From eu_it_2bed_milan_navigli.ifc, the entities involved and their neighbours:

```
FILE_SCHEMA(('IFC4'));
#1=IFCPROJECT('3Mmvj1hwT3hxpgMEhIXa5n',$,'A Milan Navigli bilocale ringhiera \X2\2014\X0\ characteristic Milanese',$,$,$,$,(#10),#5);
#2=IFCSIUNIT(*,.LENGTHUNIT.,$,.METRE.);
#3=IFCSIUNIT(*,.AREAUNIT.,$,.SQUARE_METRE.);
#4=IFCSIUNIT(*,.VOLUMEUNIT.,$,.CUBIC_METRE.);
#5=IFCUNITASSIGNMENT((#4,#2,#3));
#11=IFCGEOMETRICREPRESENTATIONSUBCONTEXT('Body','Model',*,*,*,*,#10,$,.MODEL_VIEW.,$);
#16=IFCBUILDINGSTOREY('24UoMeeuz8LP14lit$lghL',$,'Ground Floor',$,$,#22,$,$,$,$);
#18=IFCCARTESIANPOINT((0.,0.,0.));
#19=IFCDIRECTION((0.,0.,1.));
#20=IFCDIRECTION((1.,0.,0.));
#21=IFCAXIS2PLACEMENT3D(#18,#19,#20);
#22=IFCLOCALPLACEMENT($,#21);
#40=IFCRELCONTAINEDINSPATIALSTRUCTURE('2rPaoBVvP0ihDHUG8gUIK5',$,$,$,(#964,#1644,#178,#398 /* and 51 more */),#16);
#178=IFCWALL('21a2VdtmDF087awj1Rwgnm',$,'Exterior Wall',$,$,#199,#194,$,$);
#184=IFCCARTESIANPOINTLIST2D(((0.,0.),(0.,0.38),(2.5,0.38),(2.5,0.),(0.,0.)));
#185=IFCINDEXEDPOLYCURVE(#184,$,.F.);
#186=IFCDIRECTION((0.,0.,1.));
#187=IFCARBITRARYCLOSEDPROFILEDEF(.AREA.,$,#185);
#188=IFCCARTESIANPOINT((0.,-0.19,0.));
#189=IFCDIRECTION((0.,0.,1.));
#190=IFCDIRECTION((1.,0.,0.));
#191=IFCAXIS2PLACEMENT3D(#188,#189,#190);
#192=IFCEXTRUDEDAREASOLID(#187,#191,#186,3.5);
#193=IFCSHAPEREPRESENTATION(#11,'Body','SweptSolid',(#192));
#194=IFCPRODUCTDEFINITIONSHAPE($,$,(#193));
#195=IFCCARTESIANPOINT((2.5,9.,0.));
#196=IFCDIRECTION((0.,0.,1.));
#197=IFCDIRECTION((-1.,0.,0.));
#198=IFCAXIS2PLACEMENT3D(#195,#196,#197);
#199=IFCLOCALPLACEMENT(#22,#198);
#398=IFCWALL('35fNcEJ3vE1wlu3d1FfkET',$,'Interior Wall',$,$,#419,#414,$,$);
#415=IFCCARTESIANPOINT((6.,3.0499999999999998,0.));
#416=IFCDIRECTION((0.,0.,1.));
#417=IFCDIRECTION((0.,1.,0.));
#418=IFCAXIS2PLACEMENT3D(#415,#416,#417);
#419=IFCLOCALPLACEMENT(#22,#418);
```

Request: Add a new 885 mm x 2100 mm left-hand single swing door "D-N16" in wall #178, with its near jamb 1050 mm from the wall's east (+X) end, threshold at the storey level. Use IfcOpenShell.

```python
import numpy as np
import ifcopenshell
import ifcopenshell.api.feature
import ifcopenshell.api.geometry
import ifcopenshell.api.root
import ifcopenshell.api.spatial
import ifcopenshell.geom
import ifcopenshell.util.element
import ifcopenshell.util.placement
import ifcopenshell.util.representation
import ifcopenshell.util.shape
import ifcopenshell.util.unit

model = ifcopenshell.open("eu_it_2bed_milan_navigli.ifc")
unit_scale = ifcopenshell.util.unit.calculate_unit_scale(model)
settings = ifcopenshell.geom.settings()


def volume(element):
    """Net volume in cubic metres, openings subtracted."""
    shape = ifcopenshell.geom.create_shape(settings, element)
    return ifcopenshell.util.shape.get_volume(shape.geometry)


wall = model.by_id(178)
storey = ifcopenshell.util.element.get_container(wall, ifc_class="IfcBuildingStorey")
context = ifcopenshell.util.representation.get_context(model, "Model", "Body", "MODEL_VIEW")
before = volume(wall)

width, height, from_end, sill = 0.885, 2.1, 1.05, 0.0  # metres

# The wall runs along its own X axis, and the end named is its -X end.
wall_shape = ifcopenshell.geom.create_shape(settings, wall)
x, y, z = ifcopenshell.util.shape.get_vertices(wall_shape.geometry).T
start = x.min() + from_end
face, thickness = float(y.min()), float(y.max() - y.min())
wall_matrix = ifcopenshell.util.placement.get_local_placement(wall.ObjectPlacement)
level = ifcopenshell.util.placement.get_local_placement(storey.ObjectPlacement)[2, 3]


def in_wall(x, y):
    """Placement at x, y metres in the wall's axes, at sill height."""
    matrix = wall_matrix.copy()
    matrix[:, 3] = wall_matrix @ np.array([x / unit_scale, y / unit_scale, 0.0, 1.0])
    matrix[2, 3] = level + sill / unit_scale
    return matrix


# Opening: a box that overshoots both wall faces by 50 mm.
opening = ifcopenshell.api.root.create_entity(model, ifc_class="IfcOpeningElement", predefined_type="OPENING")
box = ifcopenshell.api.geometry.add_wall_representation(
    model, context=context, length=width, height=height, thickness=thickness + 0.1
)
ifcopenshell.api.geometry.assign_representation(model, product=opening, representation=box)
ifcopenshell.api.geometry.edit_object_placement(model, product=opening, matrix=in_wall(start, face - 0.05), is_si=False)
ifcopenshell.api.feature.add_feature(model, feature=opening, element=wall)

door = ifcopenshell.api.root.create_entity(model, ifc_class="IfcDoor", name="D-N16", predefined_type="DOOR")
door.OverallWidth, door.OverallHeight = width / unit_scale, height / unit_scale
door.OperationType = "SINGLE_SWING_LEFT"
body = ifcopenshell.api.geometry.add_door_representation(
    model,
    context=context,
    overall_width=door.OverallWidth,
    overall_height=door.OverallHeight,
    operation_type="SINGLE_SWING_LEFT",
    lining_properties={"LiningDepth": thickness / unit_scale, "ThresholdDepth": thickness / unit_scale},
)
ifcopenshell.api.geometry.assign_representation(model, product=door, representation=body)
ifcopenshell.api.spatial.assign_container(model, products=[door], relating_structure=storey)
ifcopenshell.api.feature.add_filling(model, opening=opening, element=door)

# The lining spans the wall, so the door starts at the wall face.
ifcopenshell.api.geometry.edit_object_placement(model, product=door, matrix=in_wall(start, face), is_si=False)

after = volume(wall)

print(f"wall volume {before:.3f} -> {after:.3f} m3")

model.write("eu_it_2bed_milan_navigli_updated.ifc")
```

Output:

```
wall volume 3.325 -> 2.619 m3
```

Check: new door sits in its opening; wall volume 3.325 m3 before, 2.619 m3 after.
